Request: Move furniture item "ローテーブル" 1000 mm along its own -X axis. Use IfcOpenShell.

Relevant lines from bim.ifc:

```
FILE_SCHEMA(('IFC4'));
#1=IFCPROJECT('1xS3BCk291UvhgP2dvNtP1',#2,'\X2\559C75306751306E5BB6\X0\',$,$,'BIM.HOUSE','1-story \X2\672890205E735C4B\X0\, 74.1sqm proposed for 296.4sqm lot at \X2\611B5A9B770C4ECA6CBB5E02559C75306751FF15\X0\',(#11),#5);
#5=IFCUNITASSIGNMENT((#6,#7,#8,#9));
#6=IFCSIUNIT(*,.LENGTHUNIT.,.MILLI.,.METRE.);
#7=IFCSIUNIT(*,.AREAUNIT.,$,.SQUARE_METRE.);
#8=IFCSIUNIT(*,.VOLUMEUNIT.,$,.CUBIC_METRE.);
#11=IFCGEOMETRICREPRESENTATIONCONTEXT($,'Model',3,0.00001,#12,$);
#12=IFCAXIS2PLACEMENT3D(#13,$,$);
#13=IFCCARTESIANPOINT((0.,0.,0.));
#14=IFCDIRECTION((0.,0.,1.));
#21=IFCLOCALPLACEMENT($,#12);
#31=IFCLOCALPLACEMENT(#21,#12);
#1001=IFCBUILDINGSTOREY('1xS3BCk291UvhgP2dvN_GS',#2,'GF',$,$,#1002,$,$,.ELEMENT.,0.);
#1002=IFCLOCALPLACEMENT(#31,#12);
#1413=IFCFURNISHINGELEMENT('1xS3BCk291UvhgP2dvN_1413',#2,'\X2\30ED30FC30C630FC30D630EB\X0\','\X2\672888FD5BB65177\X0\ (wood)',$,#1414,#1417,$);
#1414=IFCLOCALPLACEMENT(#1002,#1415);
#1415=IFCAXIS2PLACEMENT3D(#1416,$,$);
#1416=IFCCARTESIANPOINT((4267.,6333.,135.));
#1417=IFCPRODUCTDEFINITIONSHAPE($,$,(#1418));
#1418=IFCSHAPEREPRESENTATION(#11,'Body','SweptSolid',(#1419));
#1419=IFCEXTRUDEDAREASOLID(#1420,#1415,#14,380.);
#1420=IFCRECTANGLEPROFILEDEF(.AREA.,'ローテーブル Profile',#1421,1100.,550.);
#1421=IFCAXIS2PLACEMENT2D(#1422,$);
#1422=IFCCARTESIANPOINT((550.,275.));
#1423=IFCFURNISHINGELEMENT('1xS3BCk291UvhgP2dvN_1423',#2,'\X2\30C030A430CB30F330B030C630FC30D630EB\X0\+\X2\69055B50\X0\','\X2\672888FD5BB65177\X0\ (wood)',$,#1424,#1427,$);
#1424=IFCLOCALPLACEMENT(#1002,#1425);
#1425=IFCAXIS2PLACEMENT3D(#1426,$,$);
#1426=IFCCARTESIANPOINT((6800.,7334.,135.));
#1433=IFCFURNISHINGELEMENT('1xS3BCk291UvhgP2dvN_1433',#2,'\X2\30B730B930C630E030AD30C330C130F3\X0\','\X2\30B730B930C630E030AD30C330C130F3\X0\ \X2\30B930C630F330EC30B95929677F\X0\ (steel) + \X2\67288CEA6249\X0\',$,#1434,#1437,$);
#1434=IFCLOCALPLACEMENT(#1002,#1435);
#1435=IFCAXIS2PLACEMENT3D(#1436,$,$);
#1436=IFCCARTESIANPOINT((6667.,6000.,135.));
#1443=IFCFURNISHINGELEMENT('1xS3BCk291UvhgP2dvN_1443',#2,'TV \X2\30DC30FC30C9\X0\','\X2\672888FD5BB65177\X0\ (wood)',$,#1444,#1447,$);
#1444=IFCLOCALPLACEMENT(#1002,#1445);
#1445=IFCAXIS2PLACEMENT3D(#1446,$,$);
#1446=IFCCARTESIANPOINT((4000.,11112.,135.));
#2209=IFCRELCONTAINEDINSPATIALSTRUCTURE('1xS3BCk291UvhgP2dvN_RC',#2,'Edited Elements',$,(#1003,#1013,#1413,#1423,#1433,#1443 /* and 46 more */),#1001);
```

```python
import ifcopenshell
import ifcopenshell.api.geometry
import ifcopenshell.util.placement
import ifcopenshell.util.unit

model = ifcopenshell.open("bim.ifc")
unit_scale = ifcopenshell.util.unit.calculate_unit_scale(model)

item = model.by_guid("1xS3BCk291UvhgP2dvN_1413")
matrix = ifcopenshell.util.placement.get_local_placement(item.ObjectPlacement)
matrix[:3, 3] -= matrix[:3, 0] * 1 / unit_scale
ifcopenshell.api.geometry.edit_object_placement(model, product=item, matrix=matrix, is_si=False)

print(ifcopenshell.util.placement.get_local_placement(item.ObjectPlacement).round(3) + 0.0)

model.write("bim_rev.ifc")
```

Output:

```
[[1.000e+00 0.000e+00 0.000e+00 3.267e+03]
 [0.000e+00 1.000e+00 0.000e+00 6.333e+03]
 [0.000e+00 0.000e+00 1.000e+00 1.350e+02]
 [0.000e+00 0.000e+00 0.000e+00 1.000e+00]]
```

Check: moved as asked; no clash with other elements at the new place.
